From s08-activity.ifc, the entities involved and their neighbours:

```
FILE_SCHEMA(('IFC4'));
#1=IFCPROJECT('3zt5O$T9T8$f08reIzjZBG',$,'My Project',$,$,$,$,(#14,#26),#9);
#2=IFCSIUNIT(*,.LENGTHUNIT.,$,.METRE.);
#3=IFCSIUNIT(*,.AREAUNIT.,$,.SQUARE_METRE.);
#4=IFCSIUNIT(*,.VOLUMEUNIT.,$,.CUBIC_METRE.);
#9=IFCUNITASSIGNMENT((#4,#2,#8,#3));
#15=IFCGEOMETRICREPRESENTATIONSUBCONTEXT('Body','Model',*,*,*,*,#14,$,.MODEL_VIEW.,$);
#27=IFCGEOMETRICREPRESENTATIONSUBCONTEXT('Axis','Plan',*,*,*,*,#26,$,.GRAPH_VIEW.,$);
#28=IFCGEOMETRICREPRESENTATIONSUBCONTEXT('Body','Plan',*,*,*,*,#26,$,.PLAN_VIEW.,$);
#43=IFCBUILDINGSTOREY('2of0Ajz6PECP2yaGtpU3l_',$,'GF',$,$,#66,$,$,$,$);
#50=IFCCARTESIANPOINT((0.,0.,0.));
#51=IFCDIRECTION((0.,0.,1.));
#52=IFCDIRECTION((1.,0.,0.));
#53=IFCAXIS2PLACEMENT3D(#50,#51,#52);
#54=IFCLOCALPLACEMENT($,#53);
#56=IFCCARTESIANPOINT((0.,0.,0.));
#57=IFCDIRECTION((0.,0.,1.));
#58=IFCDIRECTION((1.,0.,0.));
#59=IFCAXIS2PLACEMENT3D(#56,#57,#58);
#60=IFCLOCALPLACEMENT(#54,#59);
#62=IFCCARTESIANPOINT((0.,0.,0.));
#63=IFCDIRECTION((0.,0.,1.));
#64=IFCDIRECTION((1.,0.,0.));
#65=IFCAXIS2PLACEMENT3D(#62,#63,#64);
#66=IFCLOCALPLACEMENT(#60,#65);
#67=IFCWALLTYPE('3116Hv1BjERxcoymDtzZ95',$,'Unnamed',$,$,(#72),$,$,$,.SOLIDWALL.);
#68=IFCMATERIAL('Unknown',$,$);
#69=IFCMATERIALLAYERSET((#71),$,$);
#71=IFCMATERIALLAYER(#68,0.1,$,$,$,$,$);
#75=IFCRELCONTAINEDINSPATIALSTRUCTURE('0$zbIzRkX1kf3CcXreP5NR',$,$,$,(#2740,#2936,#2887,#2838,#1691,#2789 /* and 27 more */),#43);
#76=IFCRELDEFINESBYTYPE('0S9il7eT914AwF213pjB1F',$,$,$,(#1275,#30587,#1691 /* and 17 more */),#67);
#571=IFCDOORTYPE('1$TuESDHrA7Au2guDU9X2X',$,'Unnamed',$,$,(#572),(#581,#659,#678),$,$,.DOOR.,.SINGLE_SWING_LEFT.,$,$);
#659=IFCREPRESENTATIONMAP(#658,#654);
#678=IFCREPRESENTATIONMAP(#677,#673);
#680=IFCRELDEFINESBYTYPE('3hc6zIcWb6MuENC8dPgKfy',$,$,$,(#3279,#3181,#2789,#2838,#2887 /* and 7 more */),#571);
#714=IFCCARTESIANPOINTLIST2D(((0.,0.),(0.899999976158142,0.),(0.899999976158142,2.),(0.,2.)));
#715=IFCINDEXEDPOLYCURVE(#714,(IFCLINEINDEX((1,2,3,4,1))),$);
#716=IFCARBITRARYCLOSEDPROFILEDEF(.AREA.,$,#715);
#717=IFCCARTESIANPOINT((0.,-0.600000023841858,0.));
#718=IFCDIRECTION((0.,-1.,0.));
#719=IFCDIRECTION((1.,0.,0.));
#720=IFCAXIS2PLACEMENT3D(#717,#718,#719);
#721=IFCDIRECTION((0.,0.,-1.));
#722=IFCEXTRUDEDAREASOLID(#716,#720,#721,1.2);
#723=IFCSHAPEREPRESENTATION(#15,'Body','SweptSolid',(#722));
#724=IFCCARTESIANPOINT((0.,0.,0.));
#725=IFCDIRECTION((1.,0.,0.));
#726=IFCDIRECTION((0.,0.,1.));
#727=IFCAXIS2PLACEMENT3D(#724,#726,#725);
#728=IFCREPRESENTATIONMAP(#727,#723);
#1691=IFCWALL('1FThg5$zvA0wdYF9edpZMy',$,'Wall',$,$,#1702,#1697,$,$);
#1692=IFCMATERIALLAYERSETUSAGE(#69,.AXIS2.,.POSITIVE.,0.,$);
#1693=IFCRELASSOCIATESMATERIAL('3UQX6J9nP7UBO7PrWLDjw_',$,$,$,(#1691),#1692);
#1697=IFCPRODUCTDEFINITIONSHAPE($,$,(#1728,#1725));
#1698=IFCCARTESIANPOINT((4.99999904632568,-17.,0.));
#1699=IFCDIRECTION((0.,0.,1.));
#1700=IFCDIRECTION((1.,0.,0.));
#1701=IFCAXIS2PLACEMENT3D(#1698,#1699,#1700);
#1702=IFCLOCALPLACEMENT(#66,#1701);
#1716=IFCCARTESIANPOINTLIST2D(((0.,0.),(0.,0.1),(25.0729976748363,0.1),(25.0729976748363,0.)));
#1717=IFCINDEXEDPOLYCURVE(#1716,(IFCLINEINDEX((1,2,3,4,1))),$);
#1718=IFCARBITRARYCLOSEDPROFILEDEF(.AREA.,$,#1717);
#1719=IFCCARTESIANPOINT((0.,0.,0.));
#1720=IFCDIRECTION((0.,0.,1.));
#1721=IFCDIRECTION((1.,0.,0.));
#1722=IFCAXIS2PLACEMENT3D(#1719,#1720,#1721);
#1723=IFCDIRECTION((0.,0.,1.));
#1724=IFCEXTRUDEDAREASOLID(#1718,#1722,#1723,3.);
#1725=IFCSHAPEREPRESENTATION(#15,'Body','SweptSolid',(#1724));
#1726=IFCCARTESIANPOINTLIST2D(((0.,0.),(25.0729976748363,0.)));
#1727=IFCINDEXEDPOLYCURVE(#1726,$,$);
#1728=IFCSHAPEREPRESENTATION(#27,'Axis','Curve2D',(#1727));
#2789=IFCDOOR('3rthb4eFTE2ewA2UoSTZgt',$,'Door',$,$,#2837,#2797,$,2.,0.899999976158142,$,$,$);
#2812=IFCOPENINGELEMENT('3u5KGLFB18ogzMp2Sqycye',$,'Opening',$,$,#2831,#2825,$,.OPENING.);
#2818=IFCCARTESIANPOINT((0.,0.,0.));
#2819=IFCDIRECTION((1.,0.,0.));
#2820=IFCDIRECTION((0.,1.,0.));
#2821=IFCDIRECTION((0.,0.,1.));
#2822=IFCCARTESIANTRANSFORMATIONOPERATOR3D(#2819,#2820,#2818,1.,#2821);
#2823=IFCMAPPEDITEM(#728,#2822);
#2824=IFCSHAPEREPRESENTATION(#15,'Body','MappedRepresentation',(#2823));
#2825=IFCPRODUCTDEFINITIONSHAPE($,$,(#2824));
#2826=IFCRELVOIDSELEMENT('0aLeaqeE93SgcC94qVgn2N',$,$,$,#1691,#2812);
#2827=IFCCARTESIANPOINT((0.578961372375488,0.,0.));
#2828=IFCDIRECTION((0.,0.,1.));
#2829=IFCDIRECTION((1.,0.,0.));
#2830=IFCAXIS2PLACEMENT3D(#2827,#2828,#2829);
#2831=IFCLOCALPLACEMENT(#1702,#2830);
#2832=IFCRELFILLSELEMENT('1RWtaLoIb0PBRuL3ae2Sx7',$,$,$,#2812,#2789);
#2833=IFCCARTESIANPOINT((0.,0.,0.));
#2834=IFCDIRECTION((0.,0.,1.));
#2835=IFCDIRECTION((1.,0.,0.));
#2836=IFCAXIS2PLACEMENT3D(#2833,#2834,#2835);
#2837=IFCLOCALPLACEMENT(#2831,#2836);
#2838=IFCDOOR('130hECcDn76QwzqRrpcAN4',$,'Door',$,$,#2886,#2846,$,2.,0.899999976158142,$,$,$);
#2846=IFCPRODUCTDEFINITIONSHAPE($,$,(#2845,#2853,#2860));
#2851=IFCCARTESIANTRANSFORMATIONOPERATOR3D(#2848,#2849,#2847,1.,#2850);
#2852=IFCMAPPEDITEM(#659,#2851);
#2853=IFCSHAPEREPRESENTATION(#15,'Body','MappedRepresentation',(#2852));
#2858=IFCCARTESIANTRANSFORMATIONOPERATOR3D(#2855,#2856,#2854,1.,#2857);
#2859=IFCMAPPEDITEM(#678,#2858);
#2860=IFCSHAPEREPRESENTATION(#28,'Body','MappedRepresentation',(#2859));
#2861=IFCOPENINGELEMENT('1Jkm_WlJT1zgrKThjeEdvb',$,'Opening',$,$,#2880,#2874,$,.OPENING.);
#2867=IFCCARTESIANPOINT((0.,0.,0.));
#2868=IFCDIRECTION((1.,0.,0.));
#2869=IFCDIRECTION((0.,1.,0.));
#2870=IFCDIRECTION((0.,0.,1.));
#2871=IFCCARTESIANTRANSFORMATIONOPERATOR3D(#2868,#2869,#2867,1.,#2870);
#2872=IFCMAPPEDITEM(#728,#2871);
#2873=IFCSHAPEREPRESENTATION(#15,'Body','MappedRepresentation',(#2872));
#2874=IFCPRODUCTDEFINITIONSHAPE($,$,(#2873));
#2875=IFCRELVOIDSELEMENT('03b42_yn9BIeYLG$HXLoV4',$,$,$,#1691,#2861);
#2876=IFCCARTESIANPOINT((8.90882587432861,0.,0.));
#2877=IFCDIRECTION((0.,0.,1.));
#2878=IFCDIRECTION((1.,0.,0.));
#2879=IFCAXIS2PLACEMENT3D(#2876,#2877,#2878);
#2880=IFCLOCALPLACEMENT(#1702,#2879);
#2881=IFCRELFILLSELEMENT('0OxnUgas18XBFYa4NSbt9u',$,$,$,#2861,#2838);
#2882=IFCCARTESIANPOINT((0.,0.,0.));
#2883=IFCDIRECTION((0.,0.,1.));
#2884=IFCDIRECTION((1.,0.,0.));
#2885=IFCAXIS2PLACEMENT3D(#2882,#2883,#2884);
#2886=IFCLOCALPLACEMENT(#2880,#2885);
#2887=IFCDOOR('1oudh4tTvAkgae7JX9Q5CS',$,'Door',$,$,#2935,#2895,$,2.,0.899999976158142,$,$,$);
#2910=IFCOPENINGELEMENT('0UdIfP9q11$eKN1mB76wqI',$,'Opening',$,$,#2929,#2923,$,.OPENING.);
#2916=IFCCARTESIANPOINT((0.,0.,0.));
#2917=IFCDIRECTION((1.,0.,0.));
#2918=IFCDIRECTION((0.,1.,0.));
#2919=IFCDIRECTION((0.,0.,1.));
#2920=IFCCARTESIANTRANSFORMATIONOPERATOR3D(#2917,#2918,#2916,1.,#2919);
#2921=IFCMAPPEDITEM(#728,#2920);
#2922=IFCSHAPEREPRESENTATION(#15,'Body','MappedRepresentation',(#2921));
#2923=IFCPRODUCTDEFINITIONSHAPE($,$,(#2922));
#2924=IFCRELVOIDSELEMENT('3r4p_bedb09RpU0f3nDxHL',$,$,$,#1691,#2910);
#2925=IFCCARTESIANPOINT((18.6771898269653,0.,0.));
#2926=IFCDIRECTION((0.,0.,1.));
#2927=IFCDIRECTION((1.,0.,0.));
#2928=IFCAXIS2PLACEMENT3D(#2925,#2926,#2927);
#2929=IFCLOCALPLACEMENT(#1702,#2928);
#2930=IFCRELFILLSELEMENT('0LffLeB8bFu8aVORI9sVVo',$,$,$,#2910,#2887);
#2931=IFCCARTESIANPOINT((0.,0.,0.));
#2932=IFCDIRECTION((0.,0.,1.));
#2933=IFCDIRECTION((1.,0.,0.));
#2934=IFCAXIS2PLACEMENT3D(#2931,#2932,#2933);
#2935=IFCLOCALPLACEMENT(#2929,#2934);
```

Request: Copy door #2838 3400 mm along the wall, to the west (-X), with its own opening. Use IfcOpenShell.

```python
import ifcopenshell
import ifcopenshell.api.feature
import ifcopenshell.api.geometry
import ifcopenshell.api.root
import ifcopenshell.geom
import ifcopenshell.util.element
import ifcopenshell.util.placement
import ifcopenshell.util.shape

model = ifcopenshell.open("s08-activity.ifc")
settings = ifcopenshell.geom.settings()


def volume(element):
    """Net volume in cubic metres, openings subtracted."""
    shape = ifcopenshell.geom.create_shape(settings, element)
    return ifcopenshell.util.shape.get_volume(shape.geometry)


door = model.by_guid("130hECcDn76QwzqRrpcAN4")
opening = door.FillsVoids[0].RelatingOpeningElement
wall = opening.VoidsElements[0].RelatingBuildingElement
before = volume(wall)
shift = ifcopenshell.util.placement.get_local_placement(wall.ObjectPlacement)[:3, 0] * -3.4

# copy_class copies the void relationship, type, container and properties, but no geometry.
new_opening = ifcopenshell.api.root.copy_class(model, product=opening)
new_opening.Representation = ifcopenshell.util.element.copy_deep(
    model, opening.Representation, exclude=["IfcGeometricRepresentationContext", "IfcRepresentationMap"]
)
new_door = ifcopenshell.api.root.copy_class(model, product=door)
new_door.Representation = ifcopenshell.util.element.copy_deep(
    model, door.Representation, exclude=["IfcGeometricRepresentationContext", "IfcRepresentationMap"]
)
ifcopenshell.api.feature.add_filling(model, opening=new_opening, element=new_door)

for old, new in ((opening, new_opening), (door, new_door)):
    matrix = ifcopenshell.util.placement.get_local_placement(old.ObjectPlacement)
    matrix[:3, 3] += shift
    ifcopenshell.api.geometry.edit_object_placement(model, product=new, matrix=matrix, is_si=False)

after = volume(wall)

print(f"wall volume {before:.3f} -> {after:.3f} m3")

model.write("s08-activity_rev.ifc")
```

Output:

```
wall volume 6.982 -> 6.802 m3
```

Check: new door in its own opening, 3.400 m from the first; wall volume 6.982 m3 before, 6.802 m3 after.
